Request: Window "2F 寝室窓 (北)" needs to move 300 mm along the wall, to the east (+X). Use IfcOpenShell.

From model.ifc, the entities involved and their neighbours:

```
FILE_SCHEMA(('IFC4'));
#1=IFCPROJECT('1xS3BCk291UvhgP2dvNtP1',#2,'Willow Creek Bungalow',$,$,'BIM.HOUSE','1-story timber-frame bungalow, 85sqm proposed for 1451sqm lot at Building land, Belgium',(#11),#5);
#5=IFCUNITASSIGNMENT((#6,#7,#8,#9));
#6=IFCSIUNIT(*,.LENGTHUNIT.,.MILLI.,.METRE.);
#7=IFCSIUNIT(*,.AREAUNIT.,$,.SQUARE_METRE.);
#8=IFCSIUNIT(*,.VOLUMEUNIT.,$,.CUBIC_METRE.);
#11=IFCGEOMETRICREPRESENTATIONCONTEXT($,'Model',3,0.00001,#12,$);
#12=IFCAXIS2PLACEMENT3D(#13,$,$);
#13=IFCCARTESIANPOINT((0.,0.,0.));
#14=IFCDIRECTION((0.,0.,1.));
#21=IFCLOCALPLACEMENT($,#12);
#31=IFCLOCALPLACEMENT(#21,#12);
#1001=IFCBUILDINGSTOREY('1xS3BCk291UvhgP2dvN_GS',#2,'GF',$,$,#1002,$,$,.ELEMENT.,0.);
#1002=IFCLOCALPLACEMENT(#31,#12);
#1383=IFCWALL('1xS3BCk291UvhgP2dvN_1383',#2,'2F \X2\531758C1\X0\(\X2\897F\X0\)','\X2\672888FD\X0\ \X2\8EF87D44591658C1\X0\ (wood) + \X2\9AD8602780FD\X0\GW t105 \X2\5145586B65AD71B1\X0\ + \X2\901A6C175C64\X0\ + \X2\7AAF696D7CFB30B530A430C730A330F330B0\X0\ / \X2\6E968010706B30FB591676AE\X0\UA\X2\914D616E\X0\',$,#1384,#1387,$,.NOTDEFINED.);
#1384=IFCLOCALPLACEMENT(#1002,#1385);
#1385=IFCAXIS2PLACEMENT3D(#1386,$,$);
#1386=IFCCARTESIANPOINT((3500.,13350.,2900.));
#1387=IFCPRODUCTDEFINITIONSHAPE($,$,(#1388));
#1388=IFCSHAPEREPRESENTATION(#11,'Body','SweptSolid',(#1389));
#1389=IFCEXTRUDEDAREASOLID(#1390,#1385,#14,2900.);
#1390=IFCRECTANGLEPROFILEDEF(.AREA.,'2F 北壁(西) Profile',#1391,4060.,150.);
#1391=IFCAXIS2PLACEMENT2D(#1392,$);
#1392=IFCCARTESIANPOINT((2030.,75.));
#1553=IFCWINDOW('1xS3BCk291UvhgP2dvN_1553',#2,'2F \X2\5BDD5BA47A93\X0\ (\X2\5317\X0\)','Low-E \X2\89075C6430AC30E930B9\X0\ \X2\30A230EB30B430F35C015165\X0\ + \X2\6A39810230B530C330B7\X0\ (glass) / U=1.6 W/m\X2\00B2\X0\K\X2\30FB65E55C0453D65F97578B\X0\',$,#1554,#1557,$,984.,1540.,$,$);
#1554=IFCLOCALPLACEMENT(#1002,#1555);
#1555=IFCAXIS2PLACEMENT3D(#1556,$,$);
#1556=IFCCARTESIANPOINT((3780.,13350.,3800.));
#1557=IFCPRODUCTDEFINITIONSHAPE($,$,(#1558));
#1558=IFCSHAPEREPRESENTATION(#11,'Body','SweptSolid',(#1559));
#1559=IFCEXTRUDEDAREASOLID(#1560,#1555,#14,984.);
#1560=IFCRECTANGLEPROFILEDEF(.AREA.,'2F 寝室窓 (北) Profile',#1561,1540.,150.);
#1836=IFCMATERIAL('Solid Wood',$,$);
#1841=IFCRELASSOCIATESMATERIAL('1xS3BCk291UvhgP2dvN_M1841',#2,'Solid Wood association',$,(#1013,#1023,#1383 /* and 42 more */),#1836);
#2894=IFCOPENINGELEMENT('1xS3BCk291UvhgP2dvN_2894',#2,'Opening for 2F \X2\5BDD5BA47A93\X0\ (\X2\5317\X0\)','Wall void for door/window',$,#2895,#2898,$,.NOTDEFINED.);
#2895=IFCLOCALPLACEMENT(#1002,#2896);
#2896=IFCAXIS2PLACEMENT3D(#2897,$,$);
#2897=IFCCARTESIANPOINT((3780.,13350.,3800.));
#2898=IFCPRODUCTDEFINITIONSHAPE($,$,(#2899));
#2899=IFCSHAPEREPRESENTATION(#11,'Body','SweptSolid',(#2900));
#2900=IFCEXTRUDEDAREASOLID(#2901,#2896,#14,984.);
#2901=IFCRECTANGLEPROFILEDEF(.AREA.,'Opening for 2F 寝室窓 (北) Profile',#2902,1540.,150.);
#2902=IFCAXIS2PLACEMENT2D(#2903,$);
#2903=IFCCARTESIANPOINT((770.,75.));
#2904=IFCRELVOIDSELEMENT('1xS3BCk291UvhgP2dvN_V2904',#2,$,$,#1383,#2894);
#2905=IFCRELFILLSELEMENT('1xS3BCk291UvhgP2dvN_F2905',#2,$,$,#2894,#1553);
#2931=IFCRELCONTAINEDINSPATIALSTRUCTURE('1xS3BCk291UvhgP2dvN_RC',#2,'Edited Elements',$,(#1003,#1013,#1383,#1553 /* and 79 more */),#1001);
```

```python
import ifcopenshell
import ifcopenshell.api.geometry
import ifcopenshell.util.placement

model = ifcopenshell.open("model.ifc")

window = model.by_guid("1xS3BCk291UvhgP2dvN_1553")
opening = window.FillsVoids[0].RelatingOpeningElement
wall = opening.VoidsElements[0].RelatingBuildingElement

wall_matrix = ifcopenshell.util.placement.get_local_placement(wall.ObjectPlacement)
shift = wall_matrix[:3, 0] * 300.0
before = ifcopenshell.util.placement.get_local_placement(window.ObjectPlacement)[:3, 3].copy()

# The window is not placed relative to its opening, so move both.
for product in (opening, window):
    matrix = ifcopenshell.util.placement.get_local_placement(product.ObjectPlacement)
    matrix[:3, 3] += shift
    ifcopenshell.api.geometry.edit_object_placement(model, product=product, matrix=matrix, is_si=False)

after = ifcopenshell.util.placement.get_local_placement(window.ObjectPlacement)[:3, 3]
print("window moved by", (after - before).round(3) + 0.0)

model.write("model_v2.ifc")
```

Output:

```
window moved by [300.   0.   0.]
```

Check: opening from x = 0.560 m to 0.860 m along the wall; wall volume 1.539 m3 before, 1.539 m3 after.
